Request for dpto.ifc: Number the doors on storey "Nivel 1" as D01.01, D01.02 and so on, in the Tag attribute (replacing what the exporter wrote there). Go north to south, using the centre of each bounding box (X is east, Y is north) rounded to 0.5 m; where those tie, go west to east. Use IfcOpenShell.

First a look at what the model holds.

```python
import ifcopenshell
import ifcopenshell.util.element
import ifcopenshell.util.placement

model = ifcopenshell.open("dpto.ifc")
print(model.schema)
storey = next(s for s in model.by_type("IfcBuildingStorey") if s.Name == "Nivel 1")
doors = [e for e in ifcopenshell.util.element.get_decomposition(storey) if e.is_a("IfcDoor")]
for e in sorted(doors, key=lambda e: e.id()):
    origin = ifcopenshell.util.placement.get_local_placement(e.ObjectPlacement)[:3, 3]
    print(e.id(), e.Tag, e.Name, origin.round(2) + 0.0, sep=" | ")
```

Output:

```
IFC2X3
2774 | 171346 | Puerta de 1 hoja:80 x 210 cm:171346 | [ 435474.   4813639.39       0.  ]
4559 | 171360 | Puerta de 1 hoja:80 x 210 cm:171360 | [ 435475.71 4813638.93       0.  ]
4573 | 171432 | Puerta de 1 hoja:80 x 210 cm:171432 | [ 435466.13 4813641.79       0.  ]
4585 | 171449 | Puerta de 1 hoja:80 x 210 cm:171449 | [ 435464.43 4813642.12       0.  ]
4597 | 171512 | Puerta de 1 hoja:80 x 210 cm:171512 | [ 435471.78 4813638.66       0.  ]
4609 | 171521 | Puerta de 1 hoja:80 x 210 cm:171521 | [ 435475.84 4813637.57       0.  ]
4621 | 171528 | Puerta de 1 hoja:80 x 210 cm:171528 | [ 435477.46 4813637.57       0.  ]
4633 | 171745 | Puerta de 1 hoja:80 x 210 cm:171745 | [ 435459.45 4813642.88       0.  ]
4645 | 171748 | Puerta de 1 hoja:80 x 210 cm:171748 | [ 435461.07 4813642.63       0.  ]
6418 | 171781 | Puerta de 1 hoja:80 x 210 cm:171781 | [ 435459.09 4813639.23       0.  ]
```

```python
import ifcopenshell
import ifcopenshell.geom
import ifcopenshell.util.element
import ifcopenshell.util.shape

model = ifcopenshell.open("dpto.ifc")
settings = ifcopenshell.geom.settings()
settings.set("use-world-coords", True)


def centre(element):
    shape = ifcopenshell.geom.create_shape(settings, element)
    return ifcopenshell.util.shape.get_bbox_centroid(shape.geometry)


storey = next(s for s in model.by_type("IfcBuildingStorey") if s.Name == "Nivel 1")
doors = [e for e in ifcopenshell.util.element.get_decomposition(storey) if e.is_a("IfcDoor")]

# Insertion points can sit at a corner or the storey origin, so sort by the geometry (in metres).
centres = {e: centre(e) for e in doors}
doors.sort(key=lambda e: (-round(centres[e][1] / 0.5), centres[e][0]))

for i, e in enumerate(doors, start=1):
    number = f"D01.{i:02d}"
    e.Tag = number
    print(e.id(), number)

model.write("dpto_updated.ifc")
```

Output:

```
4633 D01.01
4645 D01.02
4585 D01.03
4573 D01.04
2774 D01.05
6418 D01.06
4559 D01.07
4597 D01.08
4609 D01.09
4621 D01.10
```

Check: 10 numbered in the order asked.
